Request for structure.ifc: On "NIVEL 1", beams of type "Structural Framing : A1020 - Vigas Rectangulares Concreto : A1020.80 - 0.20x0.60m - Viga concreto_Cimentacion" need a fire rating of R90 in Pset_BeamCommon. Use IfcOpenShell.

First a look at what the model holds.

```python
import ifcopenshell
import ifcopenshell.util.element

model = ifcopenshell.open("structure.ifc")
print(model.schema)
storey = next(s for s in model.by_type("IfcBuildingStorey") if s.Name == "NIVEL 1")
beams = [e for e in ifcopenshell.util.element.get_decomposition(storey) if e.is_a("IfcBeam")]
seen = {}
for e in beams:
    element_type = ifcopenshell.util.element.get_type(e)
    key = (element_type.Name if element_type != e and element_type else None, ifcopenshell.util.element.get_pset(e, "Pset_BeamCommon", "FireRating"))
    seen[key] = seen.get(key, 0) + 1
for (name, value), count in sorted(seen.items(), key=str):
    print(count, "x", name, "|", value)
```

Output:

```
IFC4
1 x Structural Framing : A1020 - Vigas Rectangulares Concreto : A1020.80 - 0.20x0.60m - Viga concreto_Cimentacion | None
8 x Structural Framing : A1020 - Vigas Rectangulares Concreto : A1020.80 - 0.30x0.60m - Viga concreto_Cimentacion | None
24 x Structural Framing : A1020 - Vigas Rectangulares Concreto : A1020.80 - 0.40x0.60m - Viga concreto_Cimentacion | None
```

```python
import ifcopenshell
import ifcopenshell.api.pset
import ifcopenshell.util.element

model = ifcopenshell.open("structure.ifc")

storey = next(s for s in model.by_type("IfcBuildingStorey") if s.Name == "NIVEL 1")
beams = [e for e in ifcopenshell.util.element.get_decomposition(storey) if e.is_a("IfcBeam")]

count = 0
for e in beams:
    element_type = ifcopenshell.util.element.get_type(e)
    if element_type in (None, e) or element_type.Name != "Structural Framing : A1020 - Vigas Rectangulares Concreto : A1020.80 - 0.20x0.60m - Viga concreto_Cimentacion":
        continue
    # add_pset returns the element's existing set when there is one.
    pset = ifcopenshell.api.pset.add_pset(model, product=e, name="Pset_BeamCommon")
    ifcopenshell.api.pset.edit_pset(model, pset=pset, properties={"FireRating": "R90"})
    count += 1

print(count, "beams updated")

model.write("structure-out.ifc")
```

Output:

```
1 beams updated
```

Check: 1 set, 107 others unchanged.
